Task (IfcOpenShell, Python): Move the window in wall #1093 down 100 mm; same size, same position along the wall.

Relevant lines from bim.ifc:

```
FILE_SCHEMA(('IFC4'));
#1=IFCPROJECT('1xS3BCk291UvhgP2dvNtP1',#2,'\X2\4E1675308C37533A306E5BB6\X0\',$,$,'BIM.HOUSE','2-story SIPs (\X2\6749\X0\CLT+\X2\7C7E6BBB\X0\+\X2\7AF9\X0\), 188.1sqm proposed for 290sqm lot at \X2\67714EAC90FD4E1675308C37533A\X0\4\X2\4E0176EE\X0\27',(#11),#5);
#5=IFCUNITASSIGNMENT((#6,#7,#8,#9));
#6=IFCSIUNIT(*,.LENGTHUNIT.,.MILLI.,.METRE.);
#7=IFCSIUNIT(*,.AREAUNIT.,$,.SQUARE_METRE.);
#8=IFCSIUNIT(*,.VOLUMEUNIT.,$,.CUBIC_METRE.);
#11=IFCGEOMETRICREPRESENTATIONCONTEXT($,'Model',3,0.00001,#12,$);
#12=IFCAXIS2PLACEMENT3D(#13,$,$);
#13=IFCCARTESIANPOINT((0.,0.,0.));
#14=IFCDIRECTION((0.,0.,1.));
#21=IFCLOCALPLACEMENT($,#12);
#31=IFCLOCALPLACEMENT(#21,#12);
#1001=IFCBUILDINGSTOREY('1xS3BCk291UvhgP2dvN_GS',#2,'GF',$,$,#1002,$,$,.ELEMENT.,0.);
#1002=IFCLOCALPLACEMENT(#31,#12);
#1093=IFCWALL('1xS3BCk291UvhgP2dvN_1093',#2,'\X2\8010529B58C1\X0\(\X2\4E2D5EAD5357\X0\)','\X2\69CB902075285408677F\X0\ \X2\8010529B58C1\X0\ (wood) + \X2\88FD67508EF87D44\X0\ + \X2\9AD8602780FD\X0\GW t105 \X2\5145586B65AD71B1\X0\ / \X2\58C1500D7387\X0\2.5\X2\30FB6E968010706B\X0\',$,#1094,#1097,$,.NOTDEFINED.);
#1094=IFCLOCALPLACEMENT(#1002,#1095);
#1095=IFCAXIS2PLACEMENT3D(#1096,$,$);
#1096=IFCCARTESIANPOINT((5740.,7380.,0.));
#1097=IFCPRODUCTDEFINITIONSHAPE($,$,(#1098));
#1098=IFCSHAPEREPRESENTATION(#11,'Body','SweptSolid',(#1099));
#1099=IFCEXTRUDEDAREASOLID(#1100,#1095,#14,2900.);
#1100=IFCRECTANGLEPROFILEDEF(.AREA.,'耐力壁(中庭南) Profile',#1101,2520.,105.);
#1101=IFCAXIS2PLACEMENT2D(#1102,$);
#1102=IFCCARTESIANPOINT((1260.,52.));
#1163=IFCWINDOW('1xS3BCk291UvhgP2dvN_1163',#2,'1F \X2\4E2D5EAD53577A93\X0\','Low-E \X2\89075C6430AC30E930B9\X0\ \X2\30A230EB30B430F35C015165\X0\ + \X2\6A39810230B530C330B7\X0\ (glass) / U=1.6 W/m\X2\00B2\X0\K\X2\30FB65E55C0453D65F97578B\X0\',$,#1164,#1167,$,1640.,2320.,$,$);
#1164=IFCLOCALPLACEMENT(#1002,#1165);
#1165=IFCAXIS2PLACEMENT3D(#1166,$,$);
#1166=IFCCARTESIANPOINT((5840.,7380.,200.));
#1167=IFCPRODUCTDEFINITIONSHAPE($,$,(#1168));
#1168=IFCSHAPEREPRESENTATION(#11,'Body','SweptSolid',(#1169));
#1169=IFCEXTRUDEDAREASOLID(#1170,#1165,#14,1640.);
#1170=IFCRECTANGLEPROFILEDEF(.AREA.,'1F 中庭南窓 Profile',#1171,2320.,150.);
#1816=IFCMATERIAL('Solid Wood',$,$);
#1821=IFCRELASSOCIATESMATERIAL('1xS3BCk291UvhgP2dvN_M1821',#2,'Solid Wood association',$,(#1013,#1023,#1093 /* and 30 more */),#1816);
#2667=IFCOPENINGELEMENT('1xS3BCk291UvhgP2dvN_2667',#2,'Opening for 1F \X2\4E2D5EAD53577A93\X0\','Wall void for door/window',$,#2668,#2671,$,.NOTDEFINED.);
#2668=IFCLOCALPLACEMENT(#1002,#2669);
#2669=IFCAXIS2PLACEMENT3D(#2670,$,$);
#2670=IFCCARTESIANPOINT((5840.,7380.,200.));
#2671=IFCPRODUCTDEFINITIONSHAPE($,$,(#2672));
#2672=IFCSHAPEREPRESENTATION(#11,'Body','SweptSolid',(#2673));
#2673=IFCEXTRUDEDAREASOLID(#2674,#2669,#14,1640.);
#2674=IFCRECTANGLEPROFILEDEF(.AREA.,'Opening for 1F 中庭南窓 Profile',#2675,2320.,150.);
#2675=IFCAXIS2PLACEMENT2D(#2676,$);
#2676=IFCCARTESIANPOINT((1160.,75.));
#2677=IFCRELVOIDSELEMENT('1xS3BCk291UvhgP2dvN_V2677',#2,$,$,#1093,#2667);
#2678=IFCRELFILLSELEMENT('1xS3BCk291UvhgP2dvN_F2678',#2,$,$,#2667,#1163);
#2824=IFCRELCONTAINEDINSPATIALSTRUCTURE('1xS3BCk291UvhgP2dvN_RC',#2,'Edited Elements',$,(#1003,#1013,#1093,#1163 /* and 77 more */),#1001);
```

```python
import numpy as np
import ifcopenshell
import ifcopenshell.api.geometry
import ifcopenshell.util.placement
import ifcopenshell.util.unit

model = ifcopenshell.open("bim.ifc")
unit_scale = ifcopenshell.util.unit.calculate_unit_scale(model)

window = model.by_guid("1xS3BCk291UvhgP2dvN_1163")
opening = window.FillsVoids[0].RelatingOpeningElement
dz = -0.1 / unit_scale

shift = np.array([0.0, 0.0, dz])
# The window is not placed relative to its opening, so move both.
for product in (opening, window):
    matrix = ifcopenshell.util.placement.get_local_placement(product.ObjectPlacement)
    matrix[:3, 3] += shift
    ifcopenshell.api.geometry.edit_object_placement(model, product=product, matrix=matrix, is_si=False)

print(f"moved by {dz * unit_scale:+.3f} m")

model.write("bim_updated.ifc")
```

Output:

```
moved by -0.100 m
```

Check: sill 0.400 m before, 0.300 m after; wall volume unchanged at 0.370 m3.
